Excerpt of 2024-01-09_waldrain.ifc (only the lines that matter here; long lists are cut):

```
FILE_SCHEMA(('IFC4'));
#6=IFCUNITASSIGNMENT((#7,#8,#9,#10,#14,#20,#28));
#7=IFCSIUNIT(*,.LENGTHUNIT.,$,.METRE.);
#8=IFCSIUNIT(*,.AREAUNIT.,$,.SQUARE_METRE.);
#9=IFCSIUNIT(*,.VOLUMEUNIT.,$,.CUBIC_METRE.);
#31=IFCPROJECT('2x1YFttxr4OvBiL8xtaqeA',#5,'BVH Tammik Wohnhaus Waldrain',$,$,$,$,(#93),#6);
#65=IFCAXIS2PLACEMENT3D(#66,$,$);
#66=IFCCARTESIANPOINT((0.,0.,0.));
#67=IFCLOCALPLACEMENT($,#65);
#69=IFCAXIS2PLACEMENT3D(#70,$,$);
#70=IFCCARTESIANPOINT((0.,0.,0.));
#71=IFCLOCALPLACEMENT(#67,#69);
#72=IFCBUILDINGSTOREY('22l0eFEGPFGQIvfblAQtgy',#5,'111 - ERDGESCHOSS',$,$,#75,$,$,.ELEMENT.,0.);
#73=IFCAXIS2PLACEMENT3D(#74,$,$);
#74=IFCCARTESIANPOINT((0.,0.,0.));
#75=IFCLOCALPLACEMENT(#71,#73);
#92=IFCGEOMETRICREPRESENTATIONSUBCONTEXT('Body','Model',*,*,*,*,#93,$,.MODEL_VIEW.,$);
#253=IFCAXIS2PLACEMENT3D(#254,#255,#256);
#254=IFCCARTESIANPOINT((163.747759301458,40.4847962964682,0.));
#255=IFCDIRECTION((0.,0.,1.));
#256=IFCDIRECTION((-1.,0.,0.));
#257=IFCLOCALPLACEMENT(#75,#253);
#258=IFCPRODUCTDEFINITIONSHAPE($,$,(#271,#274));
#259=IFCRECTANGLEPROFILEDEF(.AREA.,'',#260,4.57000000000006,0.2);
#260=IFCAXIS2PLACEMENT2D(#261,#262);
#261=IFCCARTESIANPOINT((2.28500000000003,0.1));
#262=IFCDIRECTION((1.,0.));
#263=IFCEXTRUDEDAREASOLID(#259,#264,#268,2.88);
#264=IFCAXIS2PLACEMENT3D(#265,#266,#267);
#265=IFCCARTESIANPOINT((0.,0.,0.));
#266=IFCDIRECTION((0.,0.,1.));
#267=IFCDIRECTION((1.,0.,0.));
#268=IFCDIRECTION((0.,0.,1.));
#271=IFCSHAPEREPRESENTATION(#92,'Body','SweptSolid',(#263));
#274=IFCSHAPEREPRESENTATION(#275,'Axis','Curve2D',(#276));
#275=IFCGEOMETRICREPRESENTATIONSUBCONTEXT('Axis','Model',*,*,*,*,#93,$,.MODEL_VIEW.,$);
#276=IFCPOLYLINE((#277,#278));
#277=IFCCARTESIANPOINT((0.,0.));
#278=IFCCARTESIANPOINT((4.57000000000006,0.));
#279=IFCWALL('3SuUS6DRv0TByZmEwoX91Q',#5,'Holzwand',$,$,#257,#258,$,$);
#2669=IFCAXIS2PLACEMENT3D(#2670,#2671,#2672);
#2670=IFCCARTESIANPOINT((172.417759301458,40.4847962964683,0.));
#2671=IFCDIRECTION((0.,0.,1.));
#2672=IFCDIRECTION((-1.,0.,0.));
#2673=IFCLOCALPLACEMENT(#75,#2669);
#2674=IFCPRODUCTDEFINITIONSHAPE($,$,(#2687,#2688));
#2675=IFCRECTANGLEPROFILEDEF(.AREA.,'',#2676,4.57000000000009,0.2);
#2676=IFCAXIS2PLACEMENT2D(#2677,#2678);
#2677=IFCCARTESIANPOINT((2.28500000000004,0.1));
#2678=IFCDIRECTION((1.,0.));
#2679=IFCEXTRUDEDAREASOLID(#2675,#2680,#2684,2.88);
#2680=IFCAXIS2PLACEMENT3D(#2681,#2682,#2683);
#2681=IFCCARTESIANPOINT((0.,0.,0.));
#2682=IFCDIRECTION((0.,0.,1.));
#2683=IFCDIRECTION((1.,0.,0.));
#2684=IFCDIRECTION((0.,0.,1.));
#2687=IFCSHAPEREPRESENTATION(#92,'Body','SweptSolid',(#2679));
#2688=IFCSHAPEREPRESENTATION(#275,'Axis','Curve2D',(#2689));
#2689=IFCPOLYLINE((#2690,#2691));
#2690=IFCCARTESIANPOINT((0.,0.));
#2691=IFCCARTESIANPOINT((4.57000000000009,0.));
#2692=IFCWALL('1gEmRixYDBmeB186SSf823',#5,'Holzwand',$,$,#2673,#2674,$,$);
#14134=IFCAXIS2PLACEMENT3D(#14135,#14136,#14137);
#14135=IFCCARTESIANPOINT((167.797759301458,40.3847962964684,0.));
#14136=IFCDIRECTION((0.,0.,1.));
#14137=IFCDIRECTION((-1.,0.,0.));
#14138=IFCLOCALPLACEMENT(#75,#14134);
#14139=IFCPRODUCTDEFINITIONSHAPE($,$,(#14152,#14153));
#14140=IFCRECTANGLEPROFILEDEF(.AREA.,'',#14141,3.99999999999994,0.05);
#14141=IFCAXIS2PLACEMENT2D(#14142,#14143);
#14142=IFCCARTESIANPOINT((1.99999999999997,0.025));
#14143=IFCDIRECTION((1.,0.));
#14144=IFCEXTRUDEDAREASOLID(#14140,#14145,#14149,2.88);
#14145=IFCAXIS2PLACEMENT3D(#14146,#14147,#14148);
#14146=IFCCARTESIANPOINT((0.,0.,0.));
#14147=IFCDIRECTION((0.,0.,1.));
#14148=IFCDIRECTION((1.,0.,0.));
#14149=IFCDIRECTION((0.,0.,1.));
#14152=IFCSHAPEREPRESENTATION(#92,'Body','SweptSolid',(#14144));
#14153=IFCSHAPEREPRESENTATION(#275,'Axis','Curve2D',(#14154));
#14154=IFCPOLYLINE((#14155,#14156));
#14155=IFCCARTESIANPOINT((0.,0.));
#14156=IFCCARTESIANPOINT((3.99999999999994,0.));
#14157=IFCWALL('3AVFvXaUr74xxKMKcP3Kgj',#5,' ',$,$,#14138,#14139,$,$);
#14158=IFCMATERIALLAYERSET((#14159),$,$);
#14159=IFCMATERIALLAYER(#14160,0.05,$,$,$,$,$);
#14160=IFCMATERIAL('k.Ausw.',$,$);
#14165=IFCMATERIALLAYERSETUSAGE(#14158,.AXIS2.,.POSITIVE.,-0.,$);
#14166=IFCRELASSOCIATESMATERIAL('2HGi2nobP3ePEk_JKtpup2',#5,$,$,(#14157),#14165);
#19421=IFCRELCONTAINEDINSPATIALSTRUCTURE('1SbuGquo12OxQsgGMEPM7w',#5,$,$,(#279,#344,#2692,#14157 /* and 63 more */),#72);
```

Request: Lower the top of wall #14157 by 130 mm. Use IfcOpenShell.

```python
import ifcopenshell
import ifcopenshell.geom
import ifcopenshell.util.representation
import ifcopenshell.util.shape

model = ifcopenshell.open("2024-01-09_waldrain.ifc")
settings = ifcopenshell.geom.settings()


def volume(element):
    """Net volume in cubic metres, openings subtracted."""
    shape = ifcopenshell.geom.create_shape(settings, element)
    return ifcopenshell.util.shape.get_volume(shape.geometry)


wall = model.by_id(14157)
before = volume(wall)

body = ifcopenshell.util.representation.get_representation(wall, "Model", "Body")
solid = body.Items[0]
old_height = solid.Depth
solid.Depth -= 0.13
after = volume(wall)

print(f"height {old_height:g} -> {solid.Depth:g}, volume {before:.3f} -> {after:.3f} m3")

model.write("2024-01-09_waldrain_updated.ifc")
```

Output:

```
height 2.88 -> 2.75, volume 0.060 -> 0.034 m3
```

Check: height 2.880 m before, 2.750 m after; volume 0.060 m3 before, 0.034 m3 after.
